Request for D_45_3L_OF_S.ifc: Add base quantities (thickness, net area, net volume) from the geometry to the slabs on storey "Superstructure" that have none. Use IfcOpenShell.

First a look at what the model holds.

```python
import ifcopenshell
import ifcopenshell.util.element
import ifcopenshell.util.unit

model = ifcopenshell.open("D_45_3L_OF_S.ifc")
print(model.schema)
for unit_type in ("LENGTHUNIT", "AREAUNIT", "VOLUMEUNIT"):
    print(unit_type, ifcopenshell.util.unit.calculate_unit_scale(model, unit_type))
storey = next(s for s in model.by_type("IfcBuildingStorey") if s.Name == "Superstructure")
slabs = [e for e in ifcopenshell.util.element.get_decomposition(storey) if e.is_a("IfcSlab")]
for e in sorted(slabs, key=lambda e: e.id()):
    print(e.id(), e.is_a(), e.Name, list(ifcopenshell.util.element.get_psets(e, qtos_only=True)), sep=" | ")
```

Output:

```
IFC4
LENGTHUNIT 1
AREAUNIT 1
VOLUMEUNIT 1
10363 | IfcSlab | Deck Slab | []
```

```python
import ifcopenshell
import ifcopenshell.api.pset
import ifcopenshell.geom
import ifcopenshell.util.element
import ifcopenshell.util.shape
import ifcopenshell.util.unit

model = ifcopenshell.open("D_45_3L_OF_S.ifc")
unit_scale = ifcopenshell.util.unit.calculate_unit_scale(model)
area_scale = ifcopenshell.util.unit.calculate_unit_scale(model, "AREAUNIT")
volume_scale = ifcopenshell.util.unit.calculate_unit_scale(model, "VOLUMEUNIT")
settings = ifcopenshell.geom.settings()

storey = next(s for s in model.by_type("IfcBuildingStorey") if s.Name == "Superstructure")
slabs = [e for e in ifcopenshell.util.element.get_decomposition(storey) if e.is_a("IfcSlab")]

for e in sorted(slabs, key=lambda e: e.id()):
    if ifcopenshell.util.element.get_psets(e, qtos_only=True, should_inherit=False):
        continue
    # Geometry comes back in metres, in the element's own axes.
    shape = ifcopenshell.geom.create_shape(settings, e)
    values = {
        "Width": ifcopenshell.util.shape.get_z(shape.geometry) / unit_scale,
        "NetArea": ifcopenshell.util.shape.get_footprint_area(shape.geometry) / area_scale,
        "NetVolume": ifcopenshell.util.shape.get_volume(shape.geometry) / volume_scale,
    }
    qto = ifcopenshell.api.pset.add_qto(model, product=e, name="Qto_SlabBaseQuantities")
    ifcopenshell.api.pset.edit_qto(model, qto=qto, properties=values)
    print(e.id(), {k: round(v, 3) for k, v in values.items()})

model.write("D_45_3L_OF_S-out.ifc")
```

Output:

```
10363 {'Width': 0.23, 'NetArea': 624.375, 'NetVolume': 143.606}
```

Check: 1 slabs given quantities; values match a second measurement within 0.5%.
